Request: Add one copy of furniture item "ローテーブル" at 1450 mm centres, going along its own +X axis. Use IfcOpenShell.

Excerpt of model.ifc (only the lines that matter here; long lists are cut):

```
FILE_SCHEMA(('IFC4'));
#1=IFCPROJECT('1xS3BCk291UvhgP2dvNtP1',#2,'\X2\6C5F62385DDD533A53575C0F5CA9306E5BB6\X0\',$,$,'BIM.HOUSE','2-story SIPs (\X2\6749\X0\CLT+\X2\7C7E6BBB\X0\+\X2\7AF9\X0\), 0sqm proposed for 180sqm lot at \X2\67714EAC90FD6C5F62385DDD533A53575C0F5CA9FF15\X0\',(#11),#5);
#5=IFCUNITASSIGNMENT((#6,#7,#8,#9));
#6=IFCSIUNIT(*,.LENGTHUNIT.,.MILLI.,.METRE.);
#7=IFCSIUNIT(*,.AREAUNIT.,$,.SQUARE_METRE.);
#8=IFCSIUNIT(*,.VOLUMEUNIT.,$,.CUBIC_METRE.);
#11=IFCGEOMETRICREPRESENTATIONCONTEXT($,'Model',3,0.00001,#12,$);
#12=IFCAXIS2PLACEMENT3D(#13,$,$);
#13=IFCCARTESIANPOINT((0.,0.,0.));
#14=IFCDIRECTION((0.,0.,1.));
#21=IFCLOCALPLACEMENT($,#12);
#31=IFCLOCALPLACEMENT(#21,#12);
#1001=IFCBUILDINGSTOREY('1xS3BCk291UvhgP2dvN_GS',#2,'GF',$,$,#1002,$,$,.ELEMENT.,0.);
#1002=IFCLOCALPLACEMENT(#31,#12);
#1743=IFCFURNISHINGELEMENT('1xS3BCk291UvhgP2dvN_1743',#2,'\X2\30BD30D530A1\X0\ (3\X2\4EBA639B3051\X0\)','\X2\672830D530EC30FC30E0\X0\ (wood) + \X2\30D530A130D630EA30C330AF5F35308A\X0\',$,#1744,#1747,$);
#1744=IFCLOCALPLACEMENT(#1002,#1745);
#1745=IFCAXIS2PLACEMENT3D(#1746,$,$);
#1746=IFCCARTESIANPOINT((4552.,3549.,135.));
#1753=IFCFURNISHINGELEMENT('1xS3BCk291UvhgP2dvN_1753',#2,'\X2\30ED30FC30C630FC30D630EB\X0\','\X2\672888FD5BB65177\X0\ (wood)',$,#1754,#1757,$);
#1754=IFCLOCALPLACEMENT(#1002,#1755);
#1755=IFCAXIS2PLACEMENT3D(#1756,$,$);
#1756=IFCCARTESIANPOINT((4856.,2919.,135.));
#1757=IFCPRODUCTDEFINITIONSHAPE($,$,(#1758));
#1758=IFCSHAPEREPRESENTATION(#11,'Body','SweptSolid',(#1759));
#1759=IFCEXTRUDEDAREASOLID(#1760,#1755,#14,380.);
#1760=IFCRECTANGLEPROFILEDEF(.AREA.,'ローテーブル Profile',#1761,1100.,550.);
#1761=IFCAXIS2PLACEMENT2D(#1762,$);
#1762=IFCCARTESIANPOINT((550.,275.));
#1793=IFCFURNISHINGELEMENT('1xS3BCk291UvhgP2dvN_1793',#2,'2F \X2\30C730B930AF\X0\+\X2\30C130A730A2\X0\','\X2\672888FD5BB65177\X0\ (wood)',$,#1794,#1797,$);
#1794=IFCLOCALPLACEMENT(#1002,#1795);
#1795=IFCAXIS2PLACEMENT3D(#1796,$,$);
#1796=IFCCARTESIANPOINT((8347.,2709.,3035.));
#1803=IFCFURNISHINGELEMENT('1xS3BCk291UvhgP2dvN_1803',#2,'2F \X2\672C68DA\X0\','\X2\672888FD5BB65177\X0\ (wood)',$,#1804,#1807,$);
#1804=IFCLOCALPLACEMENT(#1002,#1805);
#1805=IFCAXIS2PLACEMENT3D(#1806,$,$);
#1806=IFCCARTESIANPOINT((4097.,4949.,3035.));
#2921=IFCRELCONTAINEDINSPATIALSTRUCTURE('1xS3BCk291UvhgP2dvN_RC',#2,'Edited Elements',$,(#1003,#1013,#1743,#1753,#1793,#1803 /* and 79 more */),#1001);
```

```python
import ifcopenshell
import ifcopenshell.api.geometry
import ifcopenshell.api.root
import ifcopenshell.util.element
import ifcopenshell.util.placement
import ifcopenshell.util.unit

model = ifcopenshell.open("model.ifc")
unit_scale = ifcopenshell.util.unit.calculate_unit_scale(model)


def reuse_history(source, copy):
    """copy_class also copies each property set's owner history, people and application; keep the originals."""
    for rel in copy.IsDefinedBy:
        if rel.is_a("IfcRelDefinesByProperties") and (history := rel.RelatingPropertyDefinition.OwnerHistory):
            rel.RelatingPropertyDefinition.OwnerHistory = source.OwnerHistory
            ifcopenshell.util.element.remove_deep2(model, history)


source = model.by_guid("1xS3BCk291UvhgP2dvN_1753")
base = ifcopenshell.util.placement.get_local_placement(source.ObjectPlacement)
step = base[:3, 0] * 1.45 / unit_scale

for i in range(1, 2):
    copy = ifcopenshell.api.root.copy_class(model, product=source)
    copy.Representation = ifcopenshell.util.element.copy_deep(
        model, source.Representation, exclude=["IfcGeometricRepresentationContext", "IfcRepresentationMap"]
    )
    reuse_history(source, copy)
    matrix = base.copy()
    matrix[:3, 3] += i * step
    print("added at", matrix[:3, 3].round(3) + 0.0)
    ifcopenshell.api.geometry.edit_object_placement(model, product=copy, matrix=matrix, is_si=False)

model.write("model_rev.ifc")
```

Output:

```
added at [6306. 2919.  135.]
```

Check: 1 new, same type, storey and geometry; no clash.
